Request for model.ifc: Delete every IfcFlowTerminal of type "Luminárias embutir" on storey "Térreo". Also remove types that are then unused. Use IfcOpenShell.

First a look at what the model holds.

```python
import ifcopenshell
import ifcopenshell.util.element

model = ifcopenshell.open("model.ifc")
print(model.schema)
storey = next(s for s in model.by_type("IfcBuildingStorey") if s.Name == "Térreo")
terminals = [e for e in ifcopenshell.util.element.get_decomposition(storey) if e.is_a("IfcFlowTerminal")]
seen = {}
for e in terminals:
    element_type = ifcopenshell.util.element.get_type(e)
    name = element_type.Name if element_type not in (None, e) else None
    seen[name] = seen.get(name, 0) + 1
for name, count in sorted(seen.items(), key=str):
    print(count, "x", name)
```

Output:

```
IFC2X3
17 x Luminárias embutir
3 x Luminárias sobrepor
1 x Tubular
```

```python
import ifcopenshell
import ifcopenshell.api.root
import ifcopenshell.util.element

model = ifcopenshell.open("model.ifc")

storey = next(s for s in model.by_type("IfcBuildingStorey") if s.Name == "Térreo")
terminals = [e for e in ifcopenshell.util.element.get_decomposition(storey) if e.is_a("IfcFlowTerminal")]
targets = [e for e in terminals if (t := ifcopenshell.util.element.get_type(e)) not in (None, e) and t.Name == "Luminárias embutir"]
types = {ifcopenshell.util.element.get_type(e) for e in targets} - {None, *targets}

for e in targets:
    ifcopenshell.api.root.remove_product(model, product=e)
print(len(targets), "removed")

unused = [t for t in types if not ifcopenshell.util.element.get_types(t)]
for t in unused:
    ifcopenshell.api.root.remove_product(model, product=t)
print(len(unused), "unused types removed")

model.write("model_edited.ifc")
```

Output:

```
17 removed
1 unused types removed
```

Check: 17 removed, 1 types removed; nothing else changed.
